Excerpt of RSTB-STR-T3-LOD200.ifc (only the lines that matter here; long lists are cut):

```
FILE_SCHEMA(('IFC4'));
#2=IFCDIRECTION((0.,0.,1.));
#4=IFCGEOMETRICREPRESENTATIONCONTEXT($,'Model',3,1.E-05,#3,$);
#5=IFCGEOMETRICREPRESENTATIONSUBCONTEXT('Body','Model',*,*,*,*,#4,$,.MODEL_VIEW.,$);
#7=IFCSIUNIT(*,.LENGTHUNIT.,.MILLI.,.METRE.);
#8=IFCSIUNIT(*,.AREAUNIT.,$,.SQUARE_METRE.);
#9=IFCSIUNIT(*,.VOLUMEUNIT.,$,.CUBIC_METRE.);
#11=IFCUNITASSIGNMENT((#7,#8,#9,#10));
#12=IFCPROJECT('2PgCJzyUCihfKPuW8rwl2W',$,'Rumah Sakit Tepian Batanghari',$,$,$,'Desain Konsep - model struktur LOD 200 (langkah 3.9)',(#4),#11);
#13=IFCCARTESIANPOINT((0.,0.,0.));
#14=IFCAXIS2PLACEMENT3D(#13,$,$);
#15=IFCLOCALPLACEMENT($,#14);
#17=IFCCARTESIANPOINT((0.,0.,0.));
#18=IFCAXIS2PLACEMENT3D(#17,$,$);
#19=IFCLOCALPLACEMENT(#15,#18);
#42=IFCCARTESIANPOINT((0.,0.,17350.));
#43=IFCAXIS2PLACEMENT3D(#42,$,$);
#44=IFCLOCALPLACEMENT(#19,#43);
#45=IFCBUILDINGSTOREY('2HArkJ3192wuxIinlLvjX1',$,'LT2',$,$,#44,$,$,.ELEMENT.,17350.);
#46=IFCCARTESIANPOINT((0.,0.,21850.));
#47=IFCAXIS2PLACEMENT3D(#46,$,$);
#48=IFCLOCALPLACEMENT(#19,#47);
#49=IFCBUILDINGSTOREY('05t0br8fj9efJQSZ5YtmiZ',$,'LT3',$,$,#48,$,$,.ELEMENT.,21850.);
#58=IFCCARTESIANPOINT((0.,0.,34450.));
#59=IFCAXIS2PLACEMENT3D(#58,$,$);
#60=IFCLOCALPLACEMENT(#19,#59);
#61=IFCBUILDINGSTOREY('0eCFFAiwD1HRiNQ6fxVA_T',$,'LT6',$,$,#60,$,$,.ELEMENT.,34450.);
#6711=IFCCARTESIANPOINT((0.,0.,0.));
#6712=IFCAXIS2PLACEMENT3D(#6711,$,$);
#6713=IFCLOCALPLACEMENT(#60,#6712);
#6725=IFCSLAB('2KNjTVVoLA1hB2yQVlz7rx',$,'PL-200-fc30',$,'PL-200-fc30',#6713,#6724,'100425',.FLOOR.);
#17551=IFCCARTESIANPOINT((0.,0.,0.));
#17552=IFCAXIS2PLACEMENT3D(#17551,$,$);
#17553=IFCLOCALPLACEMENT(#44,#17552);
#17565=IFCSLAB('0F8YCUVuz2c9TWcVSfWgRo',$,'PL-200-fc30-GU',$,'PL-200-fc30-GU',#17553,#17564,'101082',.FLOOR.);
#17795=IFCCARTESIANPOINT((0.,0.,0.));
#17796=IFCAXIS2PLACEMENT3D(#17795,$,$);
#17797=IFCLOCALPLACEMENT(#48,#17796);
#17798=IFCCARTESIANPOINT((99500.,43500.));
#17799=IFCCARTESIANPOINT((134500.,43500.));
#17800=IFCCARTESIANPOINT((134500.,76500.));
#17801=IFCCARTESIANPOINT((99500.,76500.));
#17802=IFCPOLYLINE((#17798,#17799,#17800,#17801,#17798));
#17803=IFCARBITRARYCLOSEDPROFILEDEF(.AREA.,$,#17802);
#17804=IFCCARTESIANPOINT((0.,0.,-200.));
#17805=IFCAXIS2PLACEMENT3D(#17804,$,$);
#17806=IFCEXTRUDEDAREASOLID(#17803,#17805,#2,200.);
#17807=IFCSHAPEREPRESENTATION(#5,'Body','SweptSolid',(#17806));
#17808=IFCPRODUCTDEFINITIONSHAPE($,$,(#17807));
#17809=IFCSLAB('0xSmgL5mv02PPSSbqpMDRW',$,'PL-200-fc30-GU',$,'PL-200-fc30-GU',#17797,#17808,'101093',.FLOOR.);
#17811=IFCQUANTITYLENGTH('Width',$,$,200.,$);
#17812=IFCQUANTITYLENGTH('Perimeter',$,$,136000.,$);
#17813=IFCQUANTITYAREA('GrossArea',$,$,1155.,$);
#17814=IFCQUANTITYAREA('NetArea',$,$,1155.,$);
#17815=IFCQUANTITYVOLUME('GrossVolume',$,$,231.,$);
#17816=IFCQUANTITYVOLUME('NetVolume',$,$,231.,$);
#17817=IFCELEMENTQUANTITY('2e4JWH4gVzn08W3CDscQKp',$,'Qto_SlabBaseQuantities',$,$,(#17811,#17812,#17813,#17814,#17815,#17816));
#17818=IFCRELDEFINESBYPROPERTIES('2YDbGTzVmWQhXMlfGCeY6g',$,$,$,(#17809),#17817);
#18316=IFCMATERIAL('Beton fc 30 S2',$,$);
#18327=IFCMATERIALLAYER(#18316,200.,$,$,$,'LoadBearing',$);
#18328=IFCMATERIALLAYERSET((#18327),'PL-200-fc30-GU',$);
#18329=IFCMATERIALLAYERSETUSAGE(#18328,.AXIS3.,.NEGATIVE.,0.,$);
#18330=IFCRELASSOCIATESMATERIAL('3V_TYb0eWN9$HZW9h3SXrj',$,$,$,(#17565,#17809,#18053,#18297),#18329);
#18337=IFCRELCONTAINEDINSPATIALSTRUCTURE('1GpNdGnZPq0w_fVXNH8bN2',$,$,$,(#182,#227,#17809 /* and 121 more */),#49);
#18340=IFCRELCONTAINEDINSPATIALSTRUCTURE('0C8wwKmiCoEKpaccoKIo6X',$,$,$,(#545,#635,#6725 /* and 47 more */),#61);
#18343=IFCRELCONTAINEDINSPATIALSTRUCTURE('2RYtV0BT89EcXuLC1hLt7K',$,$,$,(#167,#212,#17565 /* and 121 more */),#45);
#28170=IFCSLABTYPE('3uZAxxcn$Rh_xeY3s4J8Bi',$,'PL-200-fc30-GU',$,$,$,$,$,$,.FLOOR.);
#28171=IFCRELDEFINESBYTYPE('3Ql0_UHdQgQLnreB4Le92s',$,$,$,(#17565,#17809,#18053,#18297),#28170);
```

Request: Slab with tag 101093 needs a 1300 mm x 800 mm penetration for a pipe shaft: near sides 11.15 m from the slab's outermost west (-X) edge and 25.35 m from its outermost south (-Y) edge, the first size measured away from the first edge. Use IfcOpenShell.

```python
import numpy as np
import ifcopenshell
import ifcopenshell.api.feature
import ifcopenshell.api.geometry
import ifcopenshell.api.pset
import ifcopenshell.api.root
import ifcopenshell.geom
import ifcopenshell.util.element
import ifcopenshell.util.placement
import ifcopenshell.util.representation
import ifcopenshell.util.shape
import ifcopenshell.util.unit

model = ifcopenshell.open("RSTB-STR-T3-LOD200.ifc")
unit_scale = ifcopenshell.util.unit.calculate_unit_scale(model)
area_scale = ifcopenshell.util.unit.calculate_unit_scale(model, "AREAUNIT")
volume_scale = ifcopenshell.util.unit.calculate_unit_scale(model, "VOLUMEUNIT")
settings = ifcopenshell.geom.settings()


def volume(element):
    """Net volume in cubic metres, openings subtracted."""
    shape = ifcopenshell.geom.create_shape(settings, element)
    return ifcopenshell.util.shape.get_volume(shape.geometry)


slab = model.by_id(17809)
before = volume(slab)

# Extent in the slab's own axes, in metres. The edges named are its -X and -Y sides.
slab_shape = ifcopenshell.geom.create_shape(settings, slab)
vertices = ifcopenshell.util.shape.get_vertices(slab_shape.geometry)
x_min, y_min, bottom = vertices.min(axis=0)
top = vertices[:, 2].max()

opening = ifcopenshell.api.root.create_entity(model, ifc_class="IfcOpeningElement", name="Pipe shaft opening", predefined_type="OPENING")
context = ifcopenshell.util.representation.get_context(model, "Model", "Body", "MODEL_VIEW")
width, depth = 1.3, 0.8
outline = [(0.0, 0.0), (width, 0.0), (width, depth), (0.0, depth), (0.0, 0.0)]
# Overshoot both faces by 50 mm so the cut is clean.
shape = ifcopenshell.api.geometry.add_slab_representation(
    model, context=context, depth=top - bottom + 0.1, polyline=outline
)
ifcopenshell.api.geometry.assign_representation(model, product=opening, representation=shape)

matrix = ifcopenshell.util.placement.get_local_placement(slab.ObjectPlacement)
matrix[:, 3] = matrix @ np.append(np.array([x_min + 11.15, y_min + 25.35, bottom - 0.05]) / unit_scale, 1.0)
ifcopenshell.api.geometry.edit_object_placement(model, product=opening, matrix=matrix, is_si=False)
ifcopenshell.api.feature.add_feature(model, feature=opening, element=slab)

after = volume(slab)

# Update the slab's stored quantities.
qto = model.by_id(ifcopenshell.util.element.get_pset(slab, "Qto_SlabBaseQuantities", should_inherit=False)["id"])
ifcopenshell.api.pset.edit_qto(model, qto=qto, properties={
    "NetArea": after / (top - bottom) / area_scale,
    "NetVolume": after / volume_scale,
})

print(f"slab volume {before:.3f} -> {after:.3f} m3")

model.write("RSTB-STR-T3-LOD200-out.ifc")
```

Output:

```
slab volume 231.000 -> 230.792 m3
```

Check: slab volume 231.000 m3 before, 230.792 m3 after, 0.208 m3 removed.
